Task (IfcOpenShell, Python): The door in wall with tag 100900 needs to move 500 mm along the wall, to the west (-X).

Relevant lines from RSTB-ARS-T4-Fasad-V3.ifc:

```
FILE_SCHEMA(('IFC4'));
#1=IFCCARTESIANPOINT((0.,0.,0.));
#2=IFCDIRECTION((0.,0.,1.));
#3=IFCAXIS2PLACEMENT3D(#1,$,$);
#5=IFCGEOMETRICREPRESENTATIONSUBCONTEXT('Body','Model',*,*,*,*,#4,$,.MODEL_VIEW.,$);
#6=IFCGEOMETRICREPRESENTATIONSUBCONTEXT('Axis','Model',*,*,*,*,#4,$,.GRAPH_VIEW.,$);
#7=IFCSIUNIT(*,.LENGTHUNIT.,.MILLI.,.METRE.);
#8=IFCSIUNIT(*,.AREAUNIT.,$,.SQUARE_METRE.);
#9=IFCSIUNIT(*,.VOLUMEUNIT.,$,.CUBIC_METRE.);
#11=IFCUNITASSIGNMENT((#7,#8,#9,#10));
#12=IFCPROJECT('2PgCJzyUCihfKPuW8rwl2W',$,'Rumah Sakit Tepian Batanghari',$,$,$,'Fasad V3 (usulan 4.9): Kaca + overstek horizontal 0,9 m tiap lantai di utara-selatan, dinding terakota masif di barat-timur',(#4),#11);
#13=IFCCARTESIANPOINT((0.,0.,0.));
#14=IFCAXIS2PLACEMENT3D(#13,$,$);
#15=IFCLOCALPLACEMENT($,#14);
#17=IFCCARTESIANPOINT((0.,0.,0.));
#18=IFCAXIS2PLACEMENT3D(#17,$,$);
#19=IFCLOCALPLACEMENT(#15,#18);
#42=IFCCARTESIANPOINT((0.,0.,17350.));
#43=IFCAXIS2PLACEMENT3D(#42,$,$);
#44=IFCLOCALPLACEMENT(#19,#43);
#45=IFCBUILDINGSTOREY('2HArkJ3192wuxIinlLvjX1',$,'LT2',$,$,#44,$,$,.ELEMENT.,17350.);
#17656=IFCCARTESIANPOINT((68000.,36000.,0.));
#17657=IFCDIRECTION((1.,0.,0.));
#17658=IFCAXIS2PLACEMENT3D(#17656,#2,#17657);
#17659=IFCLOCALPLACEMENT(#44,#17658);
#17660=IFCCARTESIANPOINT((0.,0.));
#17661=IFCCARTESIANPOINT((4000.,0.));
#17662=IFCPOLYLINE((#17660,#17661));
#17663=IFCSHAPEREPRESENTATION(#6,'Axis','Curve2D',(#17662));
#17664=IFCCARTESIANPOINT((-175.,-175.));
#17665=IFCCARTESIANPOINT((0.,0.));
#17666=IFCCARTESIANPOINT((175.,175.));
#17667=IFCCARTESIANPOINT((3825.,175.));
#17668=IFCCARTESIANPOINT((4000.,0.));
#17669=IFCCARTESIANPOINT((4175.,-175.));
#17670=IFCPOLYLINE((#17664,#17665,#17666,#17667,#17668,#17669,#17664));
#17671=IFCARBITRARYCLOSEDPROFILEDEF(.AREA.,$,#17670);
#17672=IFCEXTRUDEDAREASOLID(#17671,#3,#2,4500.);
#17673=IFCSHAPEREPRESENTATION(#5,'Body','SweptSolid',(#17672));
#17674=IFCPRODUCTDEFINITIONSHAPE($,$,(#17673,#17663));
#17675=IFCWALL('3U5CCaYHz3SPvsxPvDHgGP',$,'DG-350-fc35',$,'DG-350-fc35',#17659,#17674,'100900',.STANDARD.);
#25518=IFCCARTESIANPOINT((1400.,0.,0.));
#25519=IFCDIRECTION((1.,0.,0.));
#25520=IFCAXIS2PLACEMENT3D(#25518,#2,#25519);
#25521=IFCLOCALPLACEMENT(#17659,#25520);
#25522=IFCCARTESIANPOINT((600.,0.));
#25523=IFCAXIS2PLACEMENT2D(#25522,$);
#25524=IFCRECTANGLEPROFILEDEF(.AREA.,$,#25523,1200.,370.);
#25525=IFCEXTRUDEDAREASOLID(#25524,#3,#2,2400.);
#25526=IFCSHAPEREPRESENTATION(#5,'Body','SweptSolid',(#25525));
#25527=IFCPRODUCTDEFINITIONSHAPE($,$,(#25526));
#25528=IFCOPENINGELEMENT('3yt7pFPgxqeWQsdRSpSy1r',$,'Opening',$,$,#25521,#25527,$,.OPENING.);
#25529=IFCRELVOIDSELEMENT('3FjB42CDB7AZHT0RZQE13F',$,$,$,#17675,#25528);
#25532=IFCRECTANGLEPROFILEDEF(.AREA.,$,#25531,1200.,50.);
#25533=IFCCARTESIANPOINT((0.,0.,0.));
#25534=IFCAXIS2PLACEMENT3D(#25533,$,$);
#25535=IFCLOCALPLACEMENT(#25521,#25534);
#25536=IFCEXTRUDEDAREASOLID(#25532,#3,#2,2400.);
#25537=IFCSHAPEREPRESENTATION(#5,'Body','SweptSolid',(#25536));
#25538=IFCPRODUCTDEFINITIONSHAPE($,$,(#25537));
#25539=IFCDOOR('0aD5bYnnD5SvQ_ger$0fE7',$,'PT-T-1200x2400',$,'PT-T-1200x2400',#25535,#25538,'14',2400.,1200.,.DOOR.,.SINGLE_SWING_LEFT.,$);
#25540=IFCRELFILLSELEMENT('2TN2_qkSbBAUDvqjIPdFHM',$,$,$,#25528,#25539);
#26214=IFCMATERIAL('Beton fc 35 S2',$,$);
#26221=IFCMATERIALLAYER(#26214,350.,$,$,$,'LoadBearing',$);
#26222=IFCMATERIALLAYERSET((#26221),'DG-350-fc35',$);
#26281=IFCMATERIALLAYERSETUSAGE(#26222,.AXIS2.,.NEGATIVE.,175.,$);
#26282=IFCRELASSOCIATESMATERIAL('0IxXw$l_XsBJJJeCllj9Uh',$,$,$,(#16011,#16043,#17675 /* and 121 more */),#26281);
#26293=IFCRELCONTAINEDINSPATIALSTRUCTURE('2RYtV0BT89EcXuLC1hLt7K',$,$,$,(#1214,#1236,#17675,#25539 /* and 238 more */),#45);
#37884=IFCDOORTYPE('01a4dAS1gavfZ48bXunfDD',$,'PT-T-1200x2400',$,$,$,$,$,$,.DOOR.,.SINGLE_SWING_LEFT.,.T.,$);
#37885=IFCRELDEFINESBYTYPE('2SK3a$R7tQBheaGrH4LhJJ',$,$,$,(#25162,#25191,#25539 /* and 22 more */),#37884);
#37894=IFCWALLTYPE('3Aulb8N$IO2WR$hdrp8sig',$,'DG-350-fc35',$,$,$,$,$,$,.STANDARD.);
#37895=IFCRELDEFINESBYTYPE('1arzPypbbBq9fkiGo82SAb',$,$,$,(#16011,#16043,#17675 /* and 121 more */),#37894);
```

```python
import ifcopenshell
import ifcopenshell.api.geometry
import ifcopenshell.util.placement
import ifcopenshell.util.unit

model = ifcopenshell.open("RSTB-ARS-T4-Fasad-V3.ifc")
unit_scale = ifcopenshell.util.unit.calculate_unit_scale(model)

door = model.by_id(25539)
opening = door.FillsVoids[0].RelatingOpeningElement
wall = opening.VoidsElements[0].RelatingBuildingElement

wall_matrix = ifcopenshell.util.placement.get_local_placement(wall.ObjectPlacement)
shift = wall_matrix[:3, 0] * -0.5 / unit_scale
before = ifcopenshell.util.placement.get_local_placement(door.ObjectPlacement)[:3, 3].copy()

# The door is placed relative to its opening, so it follows when the opening moves.
matrix = ifcopenshell.util.placement.get_local_placement(opening.ObjectPlacement)
matrix[:3, 3] += shift
ifcopenshell.api.geometry.edit_object_placement(
    model, product=opening, matrix=matrix, is_si=False, should_transform_children=True
)

after = ifcopenshell.util.placement.get_local_placement(door.ObjectPlacement)[:3, 3]
print("door moved by", (after - before).round(3) + 0.0)

model.write("RSTB-ARS-T4-Fasad-V3-out.ifc")
```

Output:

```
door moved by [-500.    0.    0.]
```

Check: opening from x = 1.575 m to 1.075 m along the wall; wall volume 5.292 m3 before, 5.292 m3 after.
